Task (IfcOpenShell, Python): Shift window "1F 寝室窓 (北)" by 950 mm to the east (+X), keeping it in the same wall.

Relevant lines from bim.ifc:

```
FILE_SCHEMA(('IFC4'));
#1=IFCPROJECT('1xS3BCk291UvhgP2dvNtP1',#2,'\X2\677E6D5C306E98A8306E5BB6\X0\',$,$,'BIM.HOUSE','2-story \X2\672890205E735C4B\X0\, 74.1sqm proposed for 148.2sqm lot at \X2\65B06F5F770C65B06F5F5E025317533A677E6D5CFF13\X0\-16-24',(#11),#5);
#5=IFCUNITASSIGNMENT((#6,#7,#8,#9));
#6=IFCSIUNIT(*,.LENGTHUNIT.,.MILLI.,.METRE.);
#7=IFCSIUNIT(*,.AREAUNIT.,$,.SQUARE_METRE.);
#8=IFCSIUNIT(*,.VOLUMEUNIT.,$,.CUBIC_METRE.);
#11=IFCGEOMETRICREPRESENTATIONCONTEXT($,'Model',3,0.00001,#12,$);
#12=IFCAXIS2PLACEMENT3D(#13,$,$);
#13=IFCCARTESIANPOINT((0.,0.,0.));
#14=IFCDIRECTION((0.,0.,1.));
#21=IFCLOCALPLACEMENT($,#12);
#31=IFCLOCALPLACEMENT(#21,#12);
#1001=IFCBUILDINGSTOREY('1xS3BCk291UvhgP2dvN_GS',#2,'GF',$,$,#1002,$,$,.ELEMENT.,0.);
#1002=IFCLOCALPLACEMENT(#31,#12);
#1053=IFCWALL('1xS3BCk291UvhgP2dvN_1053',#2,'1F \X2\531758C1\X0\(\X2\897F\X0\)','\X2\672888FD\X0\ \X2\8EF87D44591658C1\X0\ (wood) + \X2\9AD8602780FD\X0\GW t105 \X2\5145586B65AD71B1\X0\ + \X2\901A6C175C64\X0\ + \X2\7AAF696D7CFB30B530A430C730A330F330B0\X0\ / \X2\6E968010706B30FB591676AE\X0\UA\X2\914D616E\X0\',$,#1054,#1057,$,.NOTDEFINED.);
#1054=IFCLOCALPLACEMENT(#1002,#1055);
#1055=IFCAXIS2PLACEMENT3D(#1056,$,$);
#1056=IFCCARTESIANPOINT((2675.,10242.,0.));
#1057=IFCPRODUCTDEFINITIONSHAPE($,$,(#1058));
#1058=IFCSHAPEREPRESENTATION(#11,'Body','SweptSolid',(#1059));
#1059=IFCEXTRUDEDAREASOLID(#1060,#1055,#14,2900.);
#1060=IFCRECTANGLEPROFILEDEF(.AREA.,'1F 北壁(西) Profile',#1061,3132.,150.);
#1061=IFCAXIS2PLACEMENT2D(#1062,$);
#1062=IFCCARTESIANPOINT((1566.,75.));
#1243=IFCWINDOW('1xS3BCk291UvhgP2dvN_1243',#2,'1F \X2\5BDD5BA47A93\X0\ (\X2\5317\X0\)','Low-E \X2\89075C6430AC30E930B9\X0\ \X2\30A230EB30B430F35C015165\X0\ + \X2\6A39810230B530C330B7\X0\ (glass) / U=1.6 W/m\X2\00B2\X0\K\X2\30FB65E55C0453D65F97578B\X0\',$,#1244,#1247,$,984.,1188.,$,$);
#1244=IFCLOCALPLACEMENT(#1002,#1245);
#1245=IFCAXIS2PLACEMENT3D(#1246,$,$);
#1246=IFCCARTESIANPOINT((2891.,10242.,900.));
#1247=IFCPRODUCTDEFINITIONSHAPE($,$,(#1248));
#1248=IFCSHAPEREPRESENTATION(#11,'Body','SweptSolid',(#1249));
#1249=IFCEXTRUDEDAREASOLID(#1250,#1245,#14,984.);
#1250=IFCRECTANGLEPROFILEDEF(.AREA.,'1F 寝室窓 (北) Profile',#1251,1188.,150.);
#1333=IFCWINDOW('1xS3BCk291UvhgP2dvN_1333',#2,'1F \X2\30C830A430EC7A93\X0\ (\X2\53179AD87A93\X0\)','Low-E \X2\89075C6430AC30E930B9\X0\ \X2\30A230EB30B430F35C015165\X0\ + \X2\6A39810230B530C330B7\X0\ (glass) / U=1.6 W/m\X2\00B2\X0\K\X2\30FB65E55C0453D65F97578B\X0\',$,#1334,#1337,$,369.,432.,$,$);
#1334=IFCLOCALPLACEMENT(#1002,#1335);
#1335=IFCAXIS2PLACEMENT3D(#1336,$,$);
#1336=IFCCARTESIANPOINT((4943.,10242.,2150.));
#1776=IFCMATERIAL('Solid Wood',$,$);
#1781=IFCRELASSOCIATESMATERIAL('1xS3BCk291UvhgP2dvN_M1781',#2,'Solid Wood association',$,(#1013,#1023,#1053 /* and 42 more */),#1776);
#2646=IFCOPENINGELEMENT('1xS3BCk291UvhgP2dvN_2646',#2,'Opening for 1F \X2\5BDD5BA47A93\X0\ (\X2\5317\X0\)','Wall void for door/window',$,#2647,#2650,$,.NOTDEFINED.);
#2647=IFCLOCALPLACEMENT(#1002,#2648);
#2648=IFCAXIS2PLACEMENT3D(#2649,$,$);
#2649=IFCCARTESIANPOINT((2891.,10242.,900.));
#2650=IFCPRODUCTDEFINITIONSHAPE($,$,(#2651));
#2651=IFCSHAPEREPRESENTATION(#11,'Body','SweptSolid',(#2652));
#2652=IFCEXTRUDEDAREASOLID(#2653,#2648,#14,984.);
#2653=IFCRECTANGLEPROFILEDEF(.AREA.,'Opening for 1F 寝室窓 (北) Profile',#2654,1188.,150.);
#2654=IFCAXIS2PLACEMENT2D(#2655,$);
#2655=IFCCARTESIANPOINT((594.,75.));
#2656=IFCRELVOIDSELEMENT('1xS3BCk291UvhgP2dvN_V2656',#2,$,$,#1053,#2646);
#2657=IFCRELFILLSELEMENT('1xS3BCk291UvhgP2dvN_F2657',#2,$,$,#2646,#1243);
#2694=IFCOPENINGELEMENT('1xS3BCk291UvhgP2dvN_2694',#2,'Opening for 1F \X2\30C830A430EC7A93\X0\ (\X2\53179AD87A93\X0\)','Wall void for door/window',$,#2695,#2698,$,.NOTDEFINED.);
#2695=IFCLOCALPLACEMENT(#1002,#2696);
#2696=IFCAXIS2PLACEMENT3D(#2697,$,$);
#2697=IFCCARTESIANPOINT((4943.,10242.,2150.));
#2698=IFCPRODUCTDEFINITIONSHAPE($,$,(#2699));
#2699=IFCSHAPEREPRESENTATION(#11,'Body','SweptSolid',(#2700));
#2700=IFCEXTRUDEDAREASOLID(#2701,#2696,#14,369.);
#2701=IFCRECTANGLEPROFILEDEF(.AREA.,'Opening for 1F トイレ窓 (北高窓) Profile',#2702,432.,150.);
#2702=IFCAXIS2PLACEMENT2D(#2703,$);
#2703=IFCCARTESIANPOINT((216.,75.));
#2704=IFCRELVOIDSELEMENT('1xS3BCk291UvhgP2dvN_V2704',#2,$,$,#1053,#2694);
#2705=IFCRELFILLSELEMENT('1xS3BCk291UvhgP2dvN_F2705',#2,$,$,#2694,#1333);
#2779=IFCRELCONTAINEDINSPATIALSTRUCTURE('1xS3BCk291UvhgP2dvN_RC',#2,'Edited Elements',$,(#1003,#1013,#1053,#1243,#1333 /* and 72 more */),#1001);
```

```python
import ifcopenshell
import ifcopenshell.api.geometry
import ifcopenshell.util.placement
import ifcopenshell.util.unit

model = ifcopenshell.open("bim.ifc")
unit_scale = ifcopenshell.util.unit.calculate_unit_scale(model)

window = model.by_guid("1xS3BCk291UvhgP2dvN_1243")
opening = window.FillsVoids[0].RelatingOpeningElement
wall = opening.VoidsElements[0].RelatingBuildingElement

wall_matrix = ifcopenshell.util.placement.get_local_placement(wall.ObjectPlacement)
shift = wall_matrix[:3, 0] * 0.95 / unit_scale
before = ifcopenshell.util.placement.get_local_placement(window.ObjectPlacement)[:3, 3].copy()

# The window is not placed relative to its opening, so move both.
for product in (opening, window):
    matrix = ifcopenshell.util.placement.get_local_placement(product.ObjectPlacement)
    matrix[:3, 3] += shift
    ifcopenshell.api.geometry.edit_object_placement(model, product=product, matrix=matrix, is_si=False)

after = ifcopenshell.util.placement.get_local_placement(window.ObjectPlacement)[:3, 3]
print("window moved by", (after - before).round(3) + 0.0)

model.write("bim_edited.ifc")
```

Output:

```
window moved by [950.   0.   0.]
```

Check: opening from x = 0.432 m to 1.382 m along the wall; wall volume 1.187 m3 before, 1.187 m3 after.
